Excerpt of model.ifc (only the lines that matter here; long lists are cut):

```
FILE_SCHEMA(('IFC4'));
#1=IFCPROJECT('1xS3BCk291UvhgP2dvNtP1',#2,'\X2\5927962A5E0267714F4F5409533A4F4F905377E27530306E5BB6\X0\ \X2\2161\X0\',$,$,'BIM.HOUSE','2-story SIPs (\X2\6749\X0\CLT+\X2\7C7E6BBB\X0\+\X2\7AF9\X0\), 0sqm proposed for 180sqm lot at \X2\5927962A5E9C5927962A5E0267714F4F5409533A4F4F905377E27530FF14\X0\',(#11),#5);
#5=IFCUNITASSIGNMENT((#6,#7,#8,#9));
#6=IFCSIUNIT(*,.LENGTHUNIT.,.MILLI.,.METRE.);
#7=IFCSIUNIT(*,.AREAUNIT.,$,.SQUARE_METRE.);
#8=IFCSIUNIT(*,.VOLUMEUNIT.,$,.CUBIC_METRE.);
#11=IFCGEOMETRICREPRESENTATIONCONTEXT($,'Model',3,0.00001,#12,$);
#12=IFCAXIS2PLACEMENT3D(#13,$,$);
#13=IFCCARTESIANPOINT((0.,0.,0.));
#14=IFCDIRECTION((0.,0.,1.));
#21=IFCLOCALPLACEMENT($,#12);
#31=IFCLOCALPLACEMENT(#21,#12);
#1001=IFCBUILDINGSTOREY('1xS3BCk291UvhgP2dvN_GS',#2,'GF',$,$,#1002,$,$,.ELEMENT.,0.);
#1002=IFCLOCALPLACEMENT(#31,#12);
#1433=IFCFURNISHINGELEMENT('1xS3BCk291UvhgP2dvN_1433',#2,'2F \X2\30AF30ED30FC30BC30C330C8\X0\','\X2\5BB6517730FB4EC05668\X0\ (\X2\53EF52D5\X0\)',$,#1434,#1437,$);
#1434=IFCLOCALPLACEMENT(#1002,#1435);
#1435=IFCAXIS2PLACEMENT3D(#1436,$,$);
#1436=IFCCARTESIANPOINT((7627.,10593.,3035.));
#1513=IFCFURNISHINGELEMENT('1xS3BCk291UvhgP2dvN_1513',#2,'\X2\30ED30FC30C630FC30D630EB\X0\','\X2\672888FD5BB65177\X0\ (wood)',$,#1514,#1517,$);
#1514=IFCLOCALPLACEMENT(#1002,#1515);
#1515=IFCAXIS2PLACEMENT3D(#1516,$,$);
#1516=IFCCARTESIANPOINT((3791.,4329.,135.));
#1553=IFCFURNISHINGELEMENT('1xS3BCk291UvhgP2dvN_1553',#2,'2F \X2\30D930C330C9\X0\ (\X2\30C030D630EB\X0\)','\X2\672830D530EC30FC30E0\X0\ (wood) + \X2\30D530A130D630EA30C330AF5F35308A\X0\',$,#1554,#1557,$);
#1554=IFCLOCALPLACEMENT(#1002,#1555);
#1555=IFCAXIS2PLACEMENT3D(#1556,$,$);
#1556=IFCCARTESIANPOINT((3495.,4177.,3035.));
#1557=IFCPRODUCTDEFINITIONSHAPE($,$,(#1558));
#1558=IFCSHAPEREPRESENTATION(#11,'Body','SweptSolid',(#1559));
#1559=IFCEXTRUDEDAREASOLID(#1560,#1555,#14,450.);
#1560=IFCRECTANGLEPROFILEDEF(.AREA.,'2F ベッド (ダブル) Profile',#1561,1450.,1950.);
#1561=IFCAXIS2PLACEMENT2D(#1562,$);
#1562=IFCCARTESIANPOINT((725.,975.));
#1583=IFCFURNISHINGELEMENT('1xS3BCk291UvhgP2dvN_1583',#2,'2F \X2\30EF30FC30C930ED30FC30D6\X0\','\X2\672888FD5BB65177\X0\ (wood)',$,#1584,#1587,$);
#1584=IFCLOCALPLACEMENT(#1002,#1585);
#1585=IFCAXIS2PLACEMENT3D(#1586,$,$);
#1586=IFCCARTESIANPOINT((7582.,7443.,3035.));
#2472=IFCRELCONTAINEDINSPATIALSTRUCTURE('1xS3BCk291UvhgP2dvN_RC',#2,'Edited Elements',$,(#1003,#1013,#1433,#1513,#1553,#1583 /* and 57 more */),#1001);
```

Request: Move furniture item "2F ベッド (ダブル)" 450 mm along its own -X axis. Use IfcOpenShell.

```python
import ifcopenshell
import ifcopenshell.api.geometry
import ifcopenshell.util.placement

model = ifcopenshell.open("model.ifc")

item = model.by_guid("1xS3BCk291UvhgP2dvN_1553")
matrix = ifcopenshell.util.placement.get_local_placement(item.ObjectPlacement)
matrix[:3, 3] -= matrix[:3, 0] * 450.0
ifcopenshell.api.geometry.edit_object_placement(model, product=item, matrix=matrix, is_si=False)

print(ifcopenshell.util.placement.get_local_placement(item.ObjectPlacement).round(3) + 0.0)

model.write("model_updated.ifc")
```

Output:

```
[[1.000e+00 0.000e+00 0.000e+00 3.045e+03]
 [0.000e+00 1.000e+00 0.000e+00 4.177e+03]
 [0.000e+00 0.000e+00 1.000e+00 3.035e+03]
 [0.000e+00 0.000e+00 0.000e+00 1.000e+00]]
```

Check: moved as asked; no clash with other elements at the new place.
